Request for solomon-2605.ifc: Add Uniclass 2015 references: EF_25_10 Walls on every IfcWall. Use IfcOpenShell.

First a look at what the model holds.

```python
import ifcopenshell

model = ifcopenshell.open("solomon-2605.ifc")
print(model.schema)
print("classifications:", [c.Name for c in model.by_type("IfcClassification")])
for ifc_class in ("IfcDoor", "IfcRoof", "IfcStair", "IfcWall", "IfcWindow"):
    print(ifc_class, len(model.by_type(ifc_class)))
```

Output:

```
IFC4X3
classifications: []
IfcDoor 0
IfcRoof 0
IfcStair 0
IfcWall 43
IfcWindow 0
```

```python
import ifcopenshell
import ifcopenshell.api.classification

model = ifcopenshell.open("solomon-2605.ifc")

system = ifcopenshell.api.classification.add_classification(model, classification="Uniclass 2015")

codes = {
    "IfcWall": ("EF_25_10", "Walls"),
}
for ifc_class, (code, name) in codes.items():
    products = model.by_type(ifc_class)
    ifcopenshell.api.classification.add_reference(
        model, products=products, classification=system, identification=code, name=name
    )
    print(code, len(products))

model.write("solomon-2605_updated.ifc")
```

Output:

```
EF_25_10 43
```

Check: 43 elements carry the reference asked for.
